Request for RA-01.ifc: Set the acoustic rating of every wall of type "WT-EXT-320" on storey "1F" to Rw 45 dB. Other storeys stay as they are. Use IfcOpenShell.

First a look at what the model holds.

```python
import ifcopenshell
import ifcopenshell.util.element

model = ifcopenshell.open("RA-01.ifc")
print(model.schema)
storey = next(s for s in model.by_type("IfcBuildingStorey") if s.Name == "1F")
walls = [e for e in ifcopenshell.util.element.get_decomposition(storey) if e.is_a("IfcWall")]
seen = {}
for e in walls:
    element_type = ifcopenshell.util.element.get_type(e)
    key = (element_type.Name if element_type != e and element_type else None, ifcopenshell.util.element.get_pset(e, "Pset_WallCommon", "AcousticRating"))
    seen[key] = seen.get(key, 0) + 1
for (name, value), count in sorted(seen.items(), key=str):
    print(count, "x", name, "|", value)
```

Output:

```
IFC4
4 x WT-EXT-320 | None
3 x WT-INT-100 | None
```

```python
import ifcopenshell
import ifcopenshell.api.pset
import ifcopenshell.util.element

model = ifcopenshell.open("RA-01.ifc")

storey = next(s for s in model.by_type("IfcBuildingStorey") if s.Name == "1F")
walls = [e for e in ifcopenshell.util.element.get_decomposition(storey) if e.is_a("IfcWall")]

count = 0
for e in walls:
    element_type = ifcopenshell.util.element.get_type(e)
    if element_type in (None, e) or element_type.Name != "WT-EXT-320":
        continue
    # add_pset returns the element's existing set when there is one.
    pset = ifcopenshell.api.pset.add_pset(model, product=e, name="Pset_WallCommon")
    ifcopenshell.api.pset.edit_pset(model, pset=pset, properties={"AcousticRating": "Rw 45 dB"})
    count += 1

print(count, "walls updated")

model.write("RA-01_rev.ifc")
```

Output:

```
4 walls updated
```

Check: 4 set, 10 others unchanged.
